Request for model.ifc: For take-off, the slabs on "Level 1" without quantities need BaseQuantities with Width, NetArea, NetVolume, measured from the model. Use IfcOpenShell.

First a look at what the model holds.

```python
import ifcopenshell
import ifcopenshell.util.element
import ifcopenshell.util.unit

model = ifcopenshell.open("model.ifc")
print(model.schema)
for unit_type in ("LENGTHUNIT", "AREAUNIT", "VOLUMEUNIT"):
    print(unit_type, ifcopenshell.util.unit.calculate_unit_scale(model, unit_type))
storey = next(s for s in model.by_type("IfcBuildingStorey") if s.Name == "Level 1")
slabs = [e for e in ifcopenshell.util.element.get_decomposition(storey) if e.is_a("IfcSlab")]
for e in sorted(slabs, key=lambda e: e.id()):
    print(e.id(), e.is_a(), e.Name, list(ifcopenshell.util.element.get_psets(e, qtos_only=True)), sep=" | ")
```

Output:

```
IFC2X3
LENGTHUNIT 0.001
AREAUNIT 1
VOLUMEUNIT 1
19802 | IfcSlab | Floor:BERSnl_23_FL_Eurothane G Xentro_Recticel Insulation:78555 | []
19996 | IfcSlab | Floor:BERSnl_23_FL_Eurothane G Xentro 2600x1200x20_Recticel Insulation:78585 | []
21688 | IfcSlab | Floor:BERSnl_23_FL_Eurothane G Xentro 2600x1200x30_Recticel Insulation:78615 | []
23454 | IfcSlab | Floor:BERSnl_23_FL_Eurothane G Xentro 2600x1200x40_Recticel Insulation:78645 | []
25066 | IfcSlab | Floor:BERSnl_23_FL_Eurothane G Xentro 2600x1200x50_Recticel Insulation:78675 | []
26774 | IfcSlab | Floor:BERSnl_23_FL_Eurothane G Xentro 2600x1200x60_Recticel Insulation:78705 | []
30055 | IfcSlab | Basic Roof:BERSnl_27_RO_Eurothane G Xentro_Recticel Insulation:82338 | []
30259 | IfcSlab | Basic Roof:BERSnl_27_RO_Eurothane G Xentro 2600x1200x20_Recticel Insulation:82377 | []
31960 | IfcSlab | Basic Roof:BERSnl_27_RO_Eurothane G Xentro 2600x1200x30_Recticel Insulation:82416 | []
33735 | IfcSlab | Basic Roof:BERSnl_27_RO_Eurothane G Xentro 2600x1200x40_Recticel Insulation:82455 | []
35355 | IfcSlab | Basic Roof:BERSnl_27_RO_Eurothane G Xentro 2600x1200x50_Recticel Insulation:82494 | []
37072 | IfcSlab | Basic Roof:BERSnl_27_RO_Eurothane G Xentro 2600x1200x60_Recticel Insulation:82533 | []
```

```python
import ifcopenshell
import ifcopenshell.api.pset
import ifcopenshell.geom
import ifcopenshell.util.element
import ifcopenshell.util.shape
import ifcopenshell.util.unit

model = ifcopenshell.open("model.ifc")
unit_scale = ifcopenshell.util.unit.calculate_unit_scale(model)
area_scale = ifcopenshell.util.unit.calculate_unit_scale(model, "AREAUNIT")
volume_scale = ifcopenshell.util.unit.calculate_unit_scale(model, "VOLUMEUNIT")
settings = ifcopenshell.geom.settings()

storey = next(s for s in model.by_type("IfcBuildingStorey") if s.Name == "Level 1")
slabs = [e for e in ifcopenshell.util.element.get_decomposition(storey) if e.is_a("IfcSlab")]

for e in sorted(slabs, key=lambda e: e.id()):
    if ifcopenshell.util.element.get_psets(e, qtos_only=True, should_inherit=False):
        continue
    # Geometry comes back in metres, in the element's own axes.
    shape = ifcopenshell.geom.create_shape(settings, e)
    values = {
        "Width": ifcopenshell.util.shape.get_z(shape.geometry) / unit_scale,
        "NetArea": ifcopenshell.util.shape.get_footprint_area(shape.geometry) / area_scale,
        "NetVolume": ifcopenshell.util.shape.get_volume(shape.geometry) / volume_scale,
    }
    qto = ifcopenshell.api.pset.add_qto(model, product=e, name="BaseQuantities")
    ifcopenshell.api.pset.edit_qto(model, qto=qto, properties=values)
    print(e.id(), {k: round(v, 3) for k, v in values.items()})

model.write("model_v2.ifc")
```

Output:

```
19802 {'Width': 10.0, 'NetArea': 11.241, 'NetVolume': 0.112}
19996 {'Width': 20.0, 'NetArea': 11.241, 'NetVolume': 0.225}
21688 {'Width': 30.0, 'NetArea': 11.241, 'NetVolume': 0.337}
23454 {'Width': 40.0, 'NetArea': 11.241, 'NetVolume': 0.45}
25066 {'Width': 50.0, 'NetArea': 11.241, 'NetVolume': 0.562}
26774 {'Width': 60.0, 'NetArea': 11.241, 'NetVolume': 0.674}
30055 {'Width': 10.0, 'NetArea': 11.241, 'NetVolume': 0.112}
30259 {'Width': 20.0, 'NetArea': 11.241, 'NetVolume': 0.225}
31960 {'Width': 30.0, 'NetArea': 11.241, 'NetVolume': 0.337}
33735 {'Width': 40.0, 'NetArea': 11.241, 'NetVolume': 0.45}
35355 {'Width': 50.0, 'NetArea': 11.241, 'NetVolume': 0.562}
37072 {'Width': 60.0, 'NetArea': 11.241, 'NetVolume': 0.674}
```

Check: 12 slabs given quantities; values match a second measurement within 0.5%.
